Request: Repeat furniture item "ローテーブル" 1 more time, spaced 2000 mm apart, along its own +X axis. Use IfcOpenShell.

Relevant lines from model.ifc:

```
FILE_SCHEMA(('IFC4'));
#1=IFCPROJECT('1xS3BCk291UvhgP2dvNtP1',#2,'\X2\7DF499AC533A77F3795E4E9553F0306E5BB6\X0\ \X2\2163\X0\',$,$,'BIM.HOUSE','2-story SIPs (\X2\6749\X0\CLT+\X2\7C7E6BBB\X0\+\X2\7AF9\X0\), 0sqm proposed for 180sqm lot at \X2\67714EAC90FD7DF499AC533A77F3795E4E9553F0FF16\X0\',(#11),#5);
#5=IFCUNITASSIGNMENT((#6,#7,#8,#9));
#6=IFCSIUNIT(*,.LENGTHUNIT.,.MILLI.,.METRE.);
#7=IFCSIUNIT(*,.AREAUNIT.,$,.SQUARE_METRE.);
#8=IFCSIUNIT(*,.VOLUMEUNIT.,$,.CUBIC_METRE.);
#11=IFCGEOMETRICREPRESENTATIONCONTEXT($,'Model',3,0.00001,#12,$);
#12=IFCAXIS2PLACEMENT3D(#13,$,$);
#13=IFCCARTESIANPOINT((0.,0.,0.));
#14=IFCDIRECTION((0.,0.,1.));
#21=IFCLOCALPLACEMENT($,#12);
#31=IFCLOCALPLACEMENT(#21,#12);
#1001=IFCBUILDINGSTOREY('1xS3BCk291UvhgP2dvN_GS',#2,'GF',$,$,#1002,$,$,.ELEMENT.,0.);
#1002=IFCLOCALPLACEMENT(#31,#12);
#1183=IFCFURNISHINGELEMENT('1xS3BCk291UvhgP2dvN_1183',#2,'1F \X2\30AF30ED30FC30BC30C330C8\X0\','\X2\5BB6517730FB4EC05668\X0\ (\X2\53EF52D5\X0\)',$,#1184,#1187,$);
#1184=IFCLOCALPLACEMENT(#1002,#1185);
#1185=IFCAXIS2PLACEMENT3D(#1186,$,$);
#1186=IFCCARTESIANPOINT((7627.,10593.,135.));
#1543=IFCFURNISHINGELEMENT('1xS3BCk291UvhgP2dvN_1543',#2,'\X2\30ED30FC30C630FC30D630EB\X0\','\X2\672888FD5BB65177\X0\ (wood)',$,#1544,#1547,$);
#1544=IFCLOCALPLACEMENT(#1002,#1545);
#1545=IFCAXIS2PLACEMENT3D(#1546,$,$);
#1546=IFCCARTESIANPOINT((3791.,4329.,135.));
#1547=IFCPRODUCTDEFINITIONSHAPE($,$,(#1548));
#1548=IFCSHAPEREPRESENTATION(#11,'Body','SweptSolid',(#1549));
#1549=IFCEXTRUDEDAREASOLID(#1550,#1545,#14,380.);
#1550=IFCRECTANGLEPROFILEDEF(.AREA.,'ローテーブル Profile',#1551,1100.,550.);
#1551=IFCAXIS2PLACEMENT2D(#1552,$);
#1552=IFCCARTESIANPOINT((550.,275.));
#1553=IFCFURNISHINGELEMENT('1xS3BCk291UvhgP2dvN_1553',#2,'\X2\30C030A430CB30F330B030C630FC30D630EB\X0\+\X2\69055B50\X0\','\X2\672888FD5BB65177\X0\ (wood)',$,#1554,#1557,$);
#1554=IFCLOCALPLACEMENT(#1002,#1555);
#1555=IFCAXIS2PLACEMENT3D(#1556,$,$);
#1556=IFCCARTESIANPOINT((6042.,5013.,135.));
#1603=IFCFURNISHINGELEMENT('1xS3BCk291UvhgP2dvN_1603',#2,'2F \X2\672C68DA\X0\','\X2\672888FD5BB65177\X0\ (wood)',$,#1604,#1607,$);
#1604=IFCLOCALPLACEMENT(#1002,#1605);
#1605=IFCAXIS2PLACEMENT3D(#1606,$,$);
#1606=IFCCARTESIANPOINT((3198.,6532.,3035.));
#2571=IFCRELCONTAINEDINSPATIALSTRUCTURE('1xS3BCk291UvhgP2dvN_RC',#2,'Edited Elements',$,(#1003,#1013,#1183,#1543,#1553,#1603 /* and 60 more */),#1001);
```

```python
import ifcopenshell
import ifcopenshell.api.geometry
import ifcopenshell.api.root
import ifcopenshell.util.element
import ifcopenshell.util.placement

model = ifcopenshell.open("model.ifc")


def reuse_history(source, copy):
    """copy_class also copies each property set's owner history, people and application; keep the originals."""
    for rel in copy.IsDefinedBy:
        if rel.is_a("IfcRelDefinesByProperties") and (history := rel.RelatingPropertyDefinition.OwnerHistory):
            rel.RelatingPropertyDefinition.OwnerHistory = source.OwnerHistory
            ifcopenshell.util.element.remove_deep2(model, history)


source = model.by_guid("1xS3BCk291UvhgP2dvN_1543")
base = ifcopenshell.util.placement.get_local_placement(source.ObjectPlacement)
step = base[:3, 0] * 2000.0

for i in range(1, 2):
    copy = ifcopenshell.api.root.copy_class(model, product=source)
    copy.Representation = ifcopenshell.util.element.copy_deep(
        model, source.Representation, exclude=["IfcGeometricRepresentationContext", "IfcRepresentationMap"]
    )
    reuse_history(source, copy)
    matrix = base.copy()
    matrix[:3, 3] += i * step
    print("added at", matrix[:3, 3].round(3) + 0.0)
    ifcopenshell.api.geometry.edit_object_placement(model, product=copy, matrix=matrix, is_si=False)

model.write("model_updated.ifc")
```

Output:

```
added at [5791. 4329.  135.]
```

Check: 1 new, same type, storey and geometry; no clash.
